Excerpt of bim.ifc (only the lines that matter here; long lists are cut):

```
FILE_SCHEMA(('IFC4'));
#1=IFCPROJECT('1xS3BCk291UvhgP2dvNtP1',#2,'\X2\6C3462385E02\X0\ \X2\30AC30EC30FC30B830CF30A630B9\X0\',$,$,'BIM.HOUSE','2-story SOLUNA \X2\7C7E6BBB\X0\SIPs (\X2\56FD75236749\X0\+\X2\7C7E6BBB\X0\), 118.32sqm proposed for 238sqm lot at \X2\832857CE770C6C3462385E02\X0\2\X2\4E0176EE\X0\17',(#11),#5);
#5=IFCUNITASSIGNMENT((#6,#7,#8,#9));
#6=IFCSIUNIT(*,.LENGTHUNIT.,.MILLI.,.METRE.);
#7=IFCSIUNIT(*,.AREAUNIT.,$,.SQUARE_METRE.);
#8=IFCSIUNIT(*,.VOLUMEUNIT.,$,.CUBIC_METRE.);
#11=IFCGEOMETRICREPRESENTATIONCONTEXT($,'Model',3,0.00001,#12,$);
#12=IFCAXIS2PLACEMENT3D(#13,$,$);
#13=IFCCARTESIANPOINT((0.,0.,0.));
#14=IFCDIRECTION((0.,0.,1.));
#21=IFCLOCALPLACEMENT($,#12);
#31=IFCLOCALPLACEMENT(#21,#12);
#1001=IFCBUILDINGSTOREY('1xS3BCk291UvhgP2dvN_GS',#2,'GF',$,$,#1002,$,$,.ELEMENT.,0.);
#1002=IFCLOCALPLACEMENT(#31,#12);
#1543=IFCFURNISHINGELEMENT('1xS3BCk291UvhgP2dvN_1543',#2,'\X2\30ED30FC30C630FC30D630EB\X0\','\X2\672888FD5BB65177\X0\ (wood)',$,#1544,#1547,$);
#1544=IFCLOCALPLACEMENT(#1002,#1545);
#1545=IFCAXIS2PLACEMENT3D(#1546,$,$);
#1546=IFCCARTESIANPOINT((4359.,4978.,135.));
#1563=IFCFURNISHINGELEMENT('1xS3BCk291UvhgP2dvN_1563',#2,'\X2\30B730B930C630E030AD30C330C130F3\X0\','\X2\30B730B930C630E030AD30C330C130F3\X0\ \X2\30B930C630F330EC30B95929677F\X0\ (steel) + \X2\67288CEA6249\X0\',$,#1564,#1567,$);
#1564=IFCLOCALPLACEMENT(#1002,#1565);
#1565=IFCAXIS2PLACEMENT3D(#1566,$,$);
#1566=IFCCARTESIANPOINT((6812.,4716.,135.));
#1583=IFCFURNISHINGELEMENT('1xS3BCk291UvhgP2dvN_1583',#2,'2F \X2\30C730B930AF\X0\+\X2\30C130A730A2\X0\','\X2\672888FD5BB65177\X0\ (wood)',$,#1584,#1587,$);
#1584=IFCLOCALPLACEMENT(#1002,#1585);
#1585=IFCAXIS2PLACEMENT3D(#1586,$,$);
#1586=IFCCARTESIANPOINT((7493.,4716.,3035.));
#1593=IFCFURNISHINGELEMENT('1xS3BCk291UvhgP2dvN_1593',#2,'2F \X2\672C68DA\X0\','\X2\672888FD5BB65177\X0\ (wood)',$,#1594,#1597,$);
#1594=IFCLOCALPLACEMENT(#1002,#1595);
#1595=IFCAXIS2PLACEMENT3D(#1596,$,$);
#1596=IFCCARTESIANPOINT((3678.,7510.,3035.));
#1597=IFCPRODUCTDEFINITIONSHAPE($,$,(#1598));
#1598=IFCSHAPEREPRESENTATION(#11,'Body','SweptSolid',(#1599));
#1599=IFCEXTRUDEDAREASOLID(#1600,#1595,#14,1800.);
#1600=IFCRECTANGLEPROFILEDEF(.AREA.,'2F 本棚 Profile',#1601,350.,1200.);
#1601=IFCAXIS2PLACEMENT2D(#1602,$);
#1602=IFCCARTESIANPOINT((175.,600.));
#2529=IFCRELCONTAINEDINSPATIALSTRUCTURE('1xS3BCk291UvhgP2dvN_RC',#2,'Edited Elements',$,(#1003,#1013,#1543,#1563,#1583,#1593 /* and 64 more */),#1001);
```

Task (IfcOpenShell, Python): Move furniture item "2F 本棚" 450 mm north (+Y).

```python
import ifcopenshell
import ifcopenshell.api.geometry
import ifcopenshell.util.placement
import ifcopenshell.util.unit

model = ifcopenshell.open("bim.ifc")
unit_scale = ifcopenshell.util.unit.calculate_unit_scale(model)

item = model.by_id(1593)
matrix = ifcopenshell.util.placement.get_local_placement(item.ObjectPlacement)
matrix[1, 3] += 0.45 / unit_scale
ifcopenshell.api.geometry.edit_object_placement(model, product=item, matrix=matrix, is_si=False)

print(ifcopenshell.util.placement.get_local_placement(item.ObjectPlacement).round(3) + 0.0)

model.write("bim_edited.ifc")
```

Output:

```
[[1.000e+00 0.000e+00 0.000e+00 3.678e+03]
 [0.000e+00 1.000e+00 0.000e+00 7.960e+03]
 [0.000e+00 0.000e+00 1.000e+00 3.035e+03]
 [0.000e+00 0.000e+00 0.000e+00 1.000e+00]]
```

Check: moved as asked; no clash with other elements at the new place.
